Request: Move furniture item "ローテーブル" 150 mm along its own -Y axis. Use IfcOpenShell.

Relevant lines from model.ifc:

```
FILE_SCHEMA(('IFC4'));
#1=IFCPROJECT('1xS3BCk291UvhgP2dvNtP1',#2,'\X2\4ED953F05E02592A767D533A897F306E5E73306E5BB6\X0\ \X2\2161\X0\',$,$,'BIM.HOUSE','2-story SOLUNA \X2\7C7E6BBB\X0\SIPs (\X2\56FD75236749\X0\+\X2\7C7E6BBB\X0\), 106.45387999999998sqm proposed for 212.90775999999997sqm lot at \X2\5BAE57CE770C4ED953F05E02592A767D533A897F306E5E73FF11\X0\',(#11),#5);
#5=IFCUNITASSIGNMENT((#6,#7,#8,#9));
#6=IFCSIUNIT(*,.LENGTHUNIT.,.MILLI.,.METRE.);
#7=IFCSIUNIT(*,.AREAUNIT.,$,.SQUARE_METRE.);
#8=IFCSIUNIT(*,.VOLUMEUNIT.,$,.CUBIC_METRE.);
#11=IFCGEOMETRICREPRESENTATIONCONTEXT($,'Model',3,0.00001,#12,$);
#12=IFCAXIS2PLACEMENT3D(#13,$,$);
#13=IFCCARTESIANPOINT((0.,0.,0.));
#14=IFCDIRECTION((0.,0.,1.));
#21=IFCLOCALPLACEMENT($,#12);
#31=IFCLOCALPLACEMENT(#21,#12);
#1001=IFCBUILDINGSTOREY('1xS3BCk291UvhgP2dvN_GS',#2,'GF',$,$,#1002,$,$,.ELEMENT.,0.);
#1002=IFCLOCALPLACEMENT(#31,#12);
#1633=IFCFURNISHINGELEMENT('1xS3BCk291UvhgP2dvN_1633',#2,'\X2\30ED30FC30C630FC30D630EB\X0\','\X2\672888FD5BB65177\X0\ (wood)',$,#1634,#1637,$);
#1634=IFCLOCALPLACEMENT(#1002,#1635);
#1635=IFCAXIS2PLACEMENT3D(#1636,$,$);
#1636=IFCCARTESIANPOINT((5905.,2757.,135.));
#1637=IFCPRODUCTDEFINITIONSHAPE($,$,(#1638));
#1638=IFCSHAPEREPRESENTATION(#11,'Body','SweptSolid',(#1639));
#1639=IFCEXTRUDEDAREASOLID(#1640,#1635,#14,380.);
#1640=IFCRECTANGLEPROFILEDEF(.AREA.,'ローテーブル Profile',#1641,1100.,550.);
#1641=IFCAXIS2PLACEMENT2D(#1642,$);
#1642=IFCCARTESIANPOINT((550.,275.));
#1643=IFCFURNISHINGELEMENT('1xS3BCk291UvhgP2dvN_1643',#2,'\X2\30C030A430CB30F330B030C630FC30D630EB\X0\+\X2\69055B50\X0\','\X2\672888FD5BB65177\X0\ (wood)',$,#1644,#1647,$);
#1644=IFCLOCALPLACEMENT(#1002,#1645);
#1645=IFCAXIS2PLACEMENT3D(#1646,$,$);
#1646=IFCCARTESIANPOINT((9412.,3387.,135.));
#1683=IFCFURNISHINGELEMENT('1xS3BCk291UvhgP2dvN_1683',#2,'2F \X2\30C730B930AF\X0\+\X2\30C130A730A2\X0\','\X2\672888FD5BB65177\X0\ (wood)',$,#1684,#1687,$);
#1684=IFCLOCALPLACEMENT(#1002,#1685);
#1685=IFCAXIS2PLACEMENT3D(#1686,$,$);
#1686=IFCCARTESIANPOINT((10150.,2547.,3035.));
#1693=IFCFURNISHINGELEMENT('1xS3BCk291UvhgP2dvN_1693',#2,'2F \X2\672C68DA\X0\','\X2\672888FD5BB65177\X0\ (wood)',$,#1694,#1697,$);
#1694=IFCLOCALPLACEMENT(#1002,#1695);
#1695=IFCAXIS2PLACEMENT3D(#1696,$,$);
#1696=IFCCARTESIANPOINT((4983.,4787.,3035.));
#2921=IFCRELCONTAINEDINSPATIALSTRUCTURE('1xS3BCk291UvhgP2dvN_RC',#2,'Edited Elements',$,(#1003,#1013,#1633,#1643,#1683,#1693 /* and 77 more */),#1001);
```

```python
import ifcopenshell
import ifcopenshell.api.geometry
import ifcopenshell.util.placement
import ifcopenshell.util.unit

model = ifcopenshell.open("model.ifc")
unit_scale = ifcopenshell.util.unit.calculate_unit_scale(model)

item = model.by_guid("1xS3BCk291UvhgP2dvN_1633")
matrix = ifcopenshell.util.placement.get_local_placement(item.ObjectPlacement)
matrix[:3, 3] -= matrix[:3, 1] * 0.15 / unit_scale
ifcopenshell.api.geometry.edit_object_placement(model, product=item, matrix=matrix, is_si=False)

print(ifcopenshell.util.placement.get_local_placement(item.ObjectPlacement).round(3) + 0.0)

model.write("model-out.ifc")
```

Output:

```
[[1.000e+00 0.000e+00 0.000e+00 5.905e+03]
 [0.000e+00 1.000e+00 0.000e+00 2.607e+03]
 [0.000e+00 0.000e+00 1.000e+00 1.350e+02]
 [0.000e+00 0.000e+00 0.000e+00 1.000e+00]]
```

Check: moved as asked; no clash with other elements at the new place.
